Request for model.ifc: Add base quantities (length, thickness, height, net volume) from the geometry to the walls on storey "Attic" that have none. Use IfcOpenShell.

First a look at what the model holds.

```python
import ifcopenshell
import ifcopenshell.util.element
import ifcopenshell.util.unit

model = ifcopenshell.open("model.ifc")
print(model.schema)
for unit_type in ("LENGTHUNIT", "AREAUNIT", "VOLUMEUNIT"):
    print(unit_type, ifcopenshell.util.unit.calculate_unit_scale(model, unit_type))
storey = next(s for s in model.by_type("IfcBuildingStorey") if s.Name == "Attic")
walls = [e for e in ifcopenshell.util.element.get_decomposition(storey) if e.is_a("IfcWall")]
for e in sorted(walls, key=lambda e: e.id()):
    print(e.id(), e.is_a(), e.Name, list(ifcopenshell.util.element.get_psets(e, qtos_only=True)), sep=" | ")
```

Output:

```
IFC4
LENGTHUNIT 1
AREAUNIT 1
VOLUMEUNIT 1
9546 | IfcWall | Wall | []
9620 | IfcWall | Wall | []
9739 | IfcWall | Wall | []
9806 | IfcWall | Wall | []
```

```python
import ifcopenshell
import ifcopenshell.api.pset
import ifcopenshell.geom
import ifcopenshell.util.element
import ifcopenshell.util.shape
import ifcopenshell.util.unit

model = ifcopenshell.open("model.ifc")
unit_scale = ifcopenshell.util.unit.calculate_unit_scale(model)
volume_scale = ifcopenshell.util.unit.calculate_unit_scale(model, "VOLUMEUNIT")
settings = ifcopenshell.geom.settings()

storey = next(s for s in model.by_type("IfcBuildingStorey") if s.Name == "Attic")
walls = [e for e in ifcopenshell.util.element.get_decomposition(storey) if e.is_a("IfcWall")]

for e in sorted(walls, key=lambda e: e.id()):
    if ifcopenshell.util.element.get_psets(e, qtos_only=True, should_inherit=False):
        continue
    # Geometry comes back in metres, in the element's own axes.
    shape = ifcopenshell.geom.create_shape(settings, e)
    values = {
        "Length": ifcopenshell.util.shape.get_x(shape.geometry) / unit_scale,
        "Width": ifcopenshell.util.shape.get_y(shape.geometry) / unit_scale,
        "Height": ifcopenshell.util.shape.get_z(shape.geometry) / unit_scale,
        "NetVolume": ifcopenshell.util.shape.get_volume(shape.geometry) / volume_scale,
    }
    qto = ifcopenshell.api.pset.add_qto(model, product=e, name="Qto_WallBaseQuantities")
    ifcopenshell.api.pset.edit_qto(model, qto=qto, properties=values)
    print(e.id(), {k: round(v, 3) for k, v in values.items()})

model.write("model_rev.ifc")
```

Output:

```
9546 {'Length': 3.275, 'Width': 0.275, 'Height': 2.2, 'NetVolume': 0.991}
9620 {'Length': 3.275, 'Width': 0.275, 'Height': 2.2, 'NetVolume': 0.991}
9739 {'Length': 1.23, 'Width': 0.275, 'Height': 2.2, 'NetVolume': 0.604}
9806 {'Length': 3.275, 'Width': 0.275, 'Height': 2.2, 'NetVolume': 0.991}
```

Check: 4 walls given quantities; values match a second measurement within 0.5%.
